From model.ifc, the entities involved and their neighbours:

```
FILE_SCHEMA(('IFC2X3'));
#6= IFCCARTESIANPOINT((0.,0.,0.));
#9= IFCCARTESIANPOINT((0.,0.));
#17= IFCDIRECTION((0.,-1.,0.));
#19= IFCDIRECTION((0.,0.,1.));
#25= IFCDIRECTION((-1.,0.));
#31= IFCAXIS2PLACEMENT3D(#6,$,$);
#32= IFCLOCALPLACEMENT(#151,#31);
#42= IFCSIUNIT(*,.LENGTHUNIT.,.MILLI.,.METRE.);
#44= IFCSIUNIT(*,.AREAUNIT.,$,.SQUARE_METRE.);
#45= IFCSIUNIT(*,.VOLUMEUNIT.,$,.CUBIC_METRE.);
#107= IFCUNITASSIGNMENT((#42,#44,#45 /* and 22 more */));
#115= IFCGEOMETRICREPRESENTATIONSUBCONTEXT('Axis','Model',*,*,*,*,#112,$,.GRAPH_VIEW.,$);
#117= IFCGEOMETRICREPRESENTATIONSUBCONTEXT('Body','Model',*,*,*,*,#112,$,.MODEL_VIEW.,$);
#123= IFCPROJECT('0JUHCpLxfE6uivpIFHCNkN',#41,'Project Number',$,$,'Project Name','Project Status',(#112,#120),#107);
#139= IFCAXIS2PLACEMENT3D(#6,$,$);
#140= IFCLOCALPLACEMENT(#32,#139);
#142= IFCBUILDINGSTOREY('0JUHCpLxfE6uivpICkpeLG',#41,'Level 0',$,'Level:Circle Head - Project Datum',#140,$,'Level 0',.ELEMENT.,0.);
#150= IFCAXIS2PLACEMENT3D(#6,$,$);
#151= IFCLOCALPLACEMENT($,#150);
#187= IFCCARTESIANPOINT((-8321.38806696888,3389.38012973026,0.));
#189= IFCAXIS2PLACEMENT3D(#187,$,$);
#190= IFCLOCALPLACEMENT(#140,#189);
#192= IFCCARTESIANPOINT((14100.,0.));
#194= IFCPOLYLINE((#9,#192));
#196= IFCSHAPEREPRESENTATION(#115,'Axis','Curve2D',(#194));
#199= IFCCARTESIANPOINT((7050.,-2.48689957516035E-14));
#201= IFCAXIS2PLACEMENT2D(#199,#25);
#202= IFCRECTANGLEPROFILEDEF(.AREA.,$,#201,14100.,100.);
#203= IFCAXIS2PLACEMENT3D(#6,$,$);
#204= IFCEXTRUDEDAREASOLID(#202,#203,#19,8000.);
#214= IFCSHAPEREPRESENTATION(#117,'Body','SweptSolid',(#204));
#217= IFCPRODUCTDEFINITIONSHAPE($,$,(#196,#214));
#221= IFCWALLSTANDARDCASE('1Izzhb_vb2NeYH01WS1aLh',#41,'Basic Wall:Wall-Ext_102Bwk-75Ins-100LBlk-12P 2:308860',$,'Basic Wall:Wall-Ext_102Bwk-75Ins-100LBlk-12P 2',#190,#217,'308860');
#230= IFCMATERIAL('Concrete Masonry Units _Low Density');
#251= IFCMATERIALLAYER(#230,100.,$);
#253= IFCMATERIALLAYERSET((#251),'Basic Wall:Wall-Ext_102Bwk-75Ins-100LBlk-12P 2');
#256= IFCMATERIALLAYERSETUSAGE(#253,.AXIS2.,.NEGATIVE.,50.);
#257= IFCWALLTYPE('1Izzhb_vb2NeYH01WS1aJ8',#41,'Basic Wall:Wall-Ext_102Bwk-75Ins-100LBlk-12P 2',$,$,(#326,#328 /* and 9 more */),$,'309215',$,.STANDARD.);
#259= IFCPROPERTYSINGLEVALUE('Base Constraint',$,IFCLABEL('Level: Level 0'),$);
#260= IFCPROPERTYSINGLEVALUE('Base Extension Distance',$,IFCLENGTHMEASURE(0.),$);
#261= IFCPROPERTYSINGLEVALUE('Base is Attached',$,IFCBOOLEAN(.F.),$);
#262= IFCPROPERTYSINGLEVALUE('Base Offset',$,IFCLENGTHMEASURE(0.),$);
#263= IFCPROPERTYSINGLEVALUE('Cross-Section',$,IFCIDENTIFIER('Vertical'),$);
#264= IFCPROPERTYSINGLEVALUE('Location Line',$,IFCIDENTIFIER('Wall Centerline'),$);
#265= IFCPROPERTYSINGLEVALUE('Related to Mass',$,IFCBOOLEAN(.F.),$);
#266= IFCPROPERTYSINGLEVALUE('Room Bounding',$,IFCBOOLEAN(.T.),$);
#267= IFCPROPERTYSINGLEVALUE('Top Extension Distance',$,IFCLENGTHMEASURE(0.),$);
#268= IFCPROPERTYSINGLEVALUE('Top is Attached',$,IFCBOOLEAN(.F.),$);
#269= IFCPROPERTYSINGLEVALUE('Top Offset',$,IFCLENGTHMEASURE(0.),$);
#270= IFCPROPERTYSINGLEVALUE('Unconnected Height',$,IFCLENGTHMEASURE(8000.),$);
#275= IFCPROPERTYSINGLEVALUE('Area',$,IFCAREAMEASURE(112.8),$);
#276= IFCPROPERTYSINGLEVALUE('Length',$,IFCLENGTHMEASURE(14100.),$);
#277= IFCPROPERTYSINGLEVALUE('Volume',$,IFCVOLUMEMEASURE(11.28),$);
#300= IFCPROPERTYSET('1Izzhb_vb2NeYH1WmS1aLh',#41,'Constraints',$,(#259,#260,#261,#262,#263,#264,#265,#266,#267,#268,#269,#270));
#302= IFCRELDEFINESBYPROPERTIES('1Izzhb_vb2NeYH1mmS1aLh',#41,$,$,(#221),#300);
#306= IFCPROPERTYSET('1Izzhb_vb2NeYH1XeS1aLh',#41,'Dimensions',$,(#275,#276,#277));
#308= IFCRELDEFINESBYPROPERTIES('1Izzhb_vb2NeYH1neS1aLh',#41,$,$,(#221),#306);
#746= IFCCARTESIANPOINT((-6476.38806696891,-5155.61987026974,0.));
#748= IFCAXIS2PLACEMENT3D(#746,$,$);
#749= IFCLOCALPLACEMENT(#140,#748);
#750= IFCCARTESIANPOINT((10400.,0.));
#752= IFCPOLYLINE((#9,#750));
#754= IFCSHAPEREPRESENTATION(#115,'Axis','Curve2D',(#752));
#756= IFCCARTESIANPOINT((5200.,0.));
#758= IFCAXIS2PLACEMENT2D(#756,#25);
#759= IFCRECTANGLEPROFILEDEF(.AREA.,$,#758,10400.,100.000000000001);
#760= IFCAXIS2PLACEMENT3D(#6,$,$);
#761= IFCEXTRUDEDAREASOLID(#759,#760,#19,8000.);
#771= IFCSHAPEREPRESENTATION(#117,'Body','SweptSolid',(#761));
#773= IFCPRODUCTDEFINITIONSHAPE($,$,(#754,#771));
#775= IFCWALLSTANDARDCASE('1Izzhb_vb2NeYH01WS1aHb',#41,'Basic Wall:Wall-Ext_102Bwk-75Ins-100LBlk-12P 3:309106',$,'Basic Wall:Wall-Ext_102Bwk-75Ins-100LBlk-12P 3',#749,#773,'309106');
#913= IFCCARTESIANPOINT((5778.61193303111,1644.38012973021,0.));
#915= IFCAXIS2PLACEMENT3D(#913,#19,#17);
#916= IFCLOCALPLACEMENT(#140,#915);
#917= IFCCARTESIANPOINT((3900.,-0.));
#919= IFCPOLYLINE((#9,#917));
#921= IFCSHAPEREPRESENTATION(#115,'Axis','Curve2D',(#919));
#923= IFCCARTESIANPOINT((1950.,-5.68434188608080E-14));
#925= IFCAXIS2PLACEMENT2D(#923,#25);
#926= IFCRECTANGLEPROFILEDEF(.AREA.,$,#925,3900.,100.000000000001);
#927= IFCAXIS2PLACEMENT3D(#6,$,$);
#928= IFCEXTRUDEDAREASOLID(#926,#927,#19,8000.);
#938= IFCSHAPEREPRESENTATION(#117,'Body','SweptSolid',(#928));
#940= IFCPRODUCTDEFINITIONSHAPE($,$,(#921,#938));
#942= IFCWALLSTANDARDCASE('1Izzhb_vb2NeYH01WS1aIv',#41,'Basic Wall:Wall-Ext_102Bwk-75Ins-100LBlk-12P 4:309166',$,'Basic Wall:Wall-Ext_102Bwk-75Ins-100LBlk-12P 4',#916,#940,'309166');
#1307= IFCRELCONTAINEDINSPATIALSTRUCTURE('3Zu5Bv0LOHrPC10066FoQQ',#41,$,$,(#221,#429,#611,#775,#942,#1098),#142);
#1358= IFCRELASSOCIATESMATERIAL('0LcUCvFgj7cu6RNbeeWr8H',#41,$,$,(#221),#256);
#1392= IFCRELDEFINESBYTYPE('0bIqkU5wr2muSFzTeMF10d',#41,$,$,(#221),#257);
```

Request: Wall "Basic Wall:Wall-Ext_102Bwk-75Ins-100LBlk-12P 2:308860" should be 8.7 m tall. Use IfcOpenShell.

```python
import ifcopenshell
import ifcopenshell.api.pset
import ifcopenshell.geom
import ifcopenshell.util.element
import ifcopenshell.util.representation
import ifcopenshell.util.shape
import ifcopenshell.util.unit

model = ifcopenshell.open("model.ifc")
area_scale = ifcopenshell.util.unit.calculate_unit_scale(model, "AREAUNIT")
volume_scale = ifcopenshell.util.unit.calculate_unit_scale(model, "VOLUMEUNIT")
settings = ifcopenshell.geom.settings()


def volume(element):
    """Net volume in cubic metres, openings subtracted."""
    shape = ifcopenshell.geom.create_shape(settings, element)
    return ifcopenshell.util.shape.get_volume(shape.geometry)


wall = model.by_guid("1Izzhb_vb2NeYH01WS1aLh")
before = volume(wall)

body = ifcopenshell.util.representation.get_representation(wall, "Model", "Body")
solid = body.Items[0]
old_height = solid.Depth
solid.Depth = 8700.0
after = volume(wall)
thickness = 0.1  # wall thickness in metres

# Update the stored height, areas and volumes.
pset = model.by_id(ifcopenshell.util.element.get_pset(wall, "Constraints", should_inherit=False)["id"])
ifcopenshell.api.pset.edit_pset(model, pset=pset, properties={
    "Unconnected Height": model.create_entity("IfcLengthMeasure", solid.Depth),
})
pset = model.by_id(ifcopenshell.util.element.get_pset(wall, "Dimensions", should_inherit=False)["id"])
ifcopenshell.api.pset.edit_pset(model, pset=pset, properties={
    "Area": model.create_entity("IfcAreaMeasure", after / thickness / area_scale),
    "Volume": model.create_entity("IfcVolumeMeasure", after / volume_scale),
})

print(f"height {old_height:g} -> {solid.Depth:g}, volume {before:.3f} -> {after:.3f} m3")

model.write("model_rev.ifc")
```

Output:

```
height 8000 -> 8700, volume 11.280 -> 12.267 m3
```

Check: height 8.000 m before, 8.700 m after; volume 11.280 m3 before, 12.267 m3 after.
